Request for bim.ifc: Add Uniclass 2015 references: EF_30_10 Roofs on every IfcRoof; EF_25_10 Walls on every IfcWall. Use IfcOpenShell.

First a look at what the model holds.

```python
import ifcopenshell

model = ifcopenshell.open("bim.ifc")
print(model.schema)
print("classifications:", [c.Name for c in model.by_type("IfcClassification")])
for ifc_class in ("IfcDoor", "IfcRoof", "IfcStair", "IfcWall", "IfcWindow"):
    print(ifc_class, len(model.by_type(ifc_class)))
```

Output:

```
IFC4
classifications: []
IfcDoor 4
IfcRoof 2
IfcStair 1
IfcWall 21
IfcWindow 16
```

```python
import ifcopenshell
import ifcopenshell.api.classification

model = ifcopenshell.open("bim.ifc")

system = ifcopenshell.api.classification.add_classification(model, classification="Uniclass 2015")

codes = {
    "IfcRoof": ("EF_30_10", "Roofs"),
    "IfcWall": ("EF_25_10", "Walls"),
}
for ifc_class, (code, name) in codes.items():
    products = model.by_type(ifc_class)
    ifcopenshell.api.classification.add_reference(
        model, products=products, classification=system, identification=code, name=name
    )
    print(code, len(products))

model.write("bim_edited.ifc")
```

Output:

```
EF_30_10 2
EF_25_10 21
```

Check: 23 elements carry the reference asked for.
